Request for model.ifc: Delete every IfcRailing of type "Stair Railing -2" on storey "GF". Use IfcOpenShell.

First a look at what the model holds.

```python
import ifcopenshell
import ifcopenshell.util.element

model = ifcopenshell.open("model.ifc")
print(model.schema)
storey = next(s for s in model.by_type("IfcBuildingStorey") if s.Name == "GF")
railings = [e for e in ifcopenshell.util.element.get_decomposition(storey) if e.is_a("IfcRailing")]
seen = {}
for e in railings:
    element_type = ifcopenshell.util.element.get_type(e)
    name = element_type.Name if element_type not in (None, e) else None
    seen[name] = seen.get(name, 0) + 1
for name, count in sorted(seen.items(), key=str):
    print(count, "x", name)
```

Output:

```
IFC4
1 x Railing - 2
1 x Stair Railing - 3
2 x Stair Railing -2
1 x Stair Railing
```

```python
import ifcopenshell
import ifcopenshell.api.root
import ifcopenshell.util.element

model = ifcopenshell.open("model.ifc")

storey = next(s for s in model.by_type("IfcBuildingStorey") if s.Name == "GF")
railings = [e for e in ifcopenshell.util.element.get_decomposition(storey) if e.is_a("IfcRailing")]
targets = [e for e in railings if (t := ifcopenshell.util.element.get_type(e)) not in (None, e) and t.Name == "Stair Railing -2"]

for e in targets:
    ifcopenshell.api.root.remove_product(model, product=e)
print(len(targets), "removed")

model.write("model_updated.ifc")
```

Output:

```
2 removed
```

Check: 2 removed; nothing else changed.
